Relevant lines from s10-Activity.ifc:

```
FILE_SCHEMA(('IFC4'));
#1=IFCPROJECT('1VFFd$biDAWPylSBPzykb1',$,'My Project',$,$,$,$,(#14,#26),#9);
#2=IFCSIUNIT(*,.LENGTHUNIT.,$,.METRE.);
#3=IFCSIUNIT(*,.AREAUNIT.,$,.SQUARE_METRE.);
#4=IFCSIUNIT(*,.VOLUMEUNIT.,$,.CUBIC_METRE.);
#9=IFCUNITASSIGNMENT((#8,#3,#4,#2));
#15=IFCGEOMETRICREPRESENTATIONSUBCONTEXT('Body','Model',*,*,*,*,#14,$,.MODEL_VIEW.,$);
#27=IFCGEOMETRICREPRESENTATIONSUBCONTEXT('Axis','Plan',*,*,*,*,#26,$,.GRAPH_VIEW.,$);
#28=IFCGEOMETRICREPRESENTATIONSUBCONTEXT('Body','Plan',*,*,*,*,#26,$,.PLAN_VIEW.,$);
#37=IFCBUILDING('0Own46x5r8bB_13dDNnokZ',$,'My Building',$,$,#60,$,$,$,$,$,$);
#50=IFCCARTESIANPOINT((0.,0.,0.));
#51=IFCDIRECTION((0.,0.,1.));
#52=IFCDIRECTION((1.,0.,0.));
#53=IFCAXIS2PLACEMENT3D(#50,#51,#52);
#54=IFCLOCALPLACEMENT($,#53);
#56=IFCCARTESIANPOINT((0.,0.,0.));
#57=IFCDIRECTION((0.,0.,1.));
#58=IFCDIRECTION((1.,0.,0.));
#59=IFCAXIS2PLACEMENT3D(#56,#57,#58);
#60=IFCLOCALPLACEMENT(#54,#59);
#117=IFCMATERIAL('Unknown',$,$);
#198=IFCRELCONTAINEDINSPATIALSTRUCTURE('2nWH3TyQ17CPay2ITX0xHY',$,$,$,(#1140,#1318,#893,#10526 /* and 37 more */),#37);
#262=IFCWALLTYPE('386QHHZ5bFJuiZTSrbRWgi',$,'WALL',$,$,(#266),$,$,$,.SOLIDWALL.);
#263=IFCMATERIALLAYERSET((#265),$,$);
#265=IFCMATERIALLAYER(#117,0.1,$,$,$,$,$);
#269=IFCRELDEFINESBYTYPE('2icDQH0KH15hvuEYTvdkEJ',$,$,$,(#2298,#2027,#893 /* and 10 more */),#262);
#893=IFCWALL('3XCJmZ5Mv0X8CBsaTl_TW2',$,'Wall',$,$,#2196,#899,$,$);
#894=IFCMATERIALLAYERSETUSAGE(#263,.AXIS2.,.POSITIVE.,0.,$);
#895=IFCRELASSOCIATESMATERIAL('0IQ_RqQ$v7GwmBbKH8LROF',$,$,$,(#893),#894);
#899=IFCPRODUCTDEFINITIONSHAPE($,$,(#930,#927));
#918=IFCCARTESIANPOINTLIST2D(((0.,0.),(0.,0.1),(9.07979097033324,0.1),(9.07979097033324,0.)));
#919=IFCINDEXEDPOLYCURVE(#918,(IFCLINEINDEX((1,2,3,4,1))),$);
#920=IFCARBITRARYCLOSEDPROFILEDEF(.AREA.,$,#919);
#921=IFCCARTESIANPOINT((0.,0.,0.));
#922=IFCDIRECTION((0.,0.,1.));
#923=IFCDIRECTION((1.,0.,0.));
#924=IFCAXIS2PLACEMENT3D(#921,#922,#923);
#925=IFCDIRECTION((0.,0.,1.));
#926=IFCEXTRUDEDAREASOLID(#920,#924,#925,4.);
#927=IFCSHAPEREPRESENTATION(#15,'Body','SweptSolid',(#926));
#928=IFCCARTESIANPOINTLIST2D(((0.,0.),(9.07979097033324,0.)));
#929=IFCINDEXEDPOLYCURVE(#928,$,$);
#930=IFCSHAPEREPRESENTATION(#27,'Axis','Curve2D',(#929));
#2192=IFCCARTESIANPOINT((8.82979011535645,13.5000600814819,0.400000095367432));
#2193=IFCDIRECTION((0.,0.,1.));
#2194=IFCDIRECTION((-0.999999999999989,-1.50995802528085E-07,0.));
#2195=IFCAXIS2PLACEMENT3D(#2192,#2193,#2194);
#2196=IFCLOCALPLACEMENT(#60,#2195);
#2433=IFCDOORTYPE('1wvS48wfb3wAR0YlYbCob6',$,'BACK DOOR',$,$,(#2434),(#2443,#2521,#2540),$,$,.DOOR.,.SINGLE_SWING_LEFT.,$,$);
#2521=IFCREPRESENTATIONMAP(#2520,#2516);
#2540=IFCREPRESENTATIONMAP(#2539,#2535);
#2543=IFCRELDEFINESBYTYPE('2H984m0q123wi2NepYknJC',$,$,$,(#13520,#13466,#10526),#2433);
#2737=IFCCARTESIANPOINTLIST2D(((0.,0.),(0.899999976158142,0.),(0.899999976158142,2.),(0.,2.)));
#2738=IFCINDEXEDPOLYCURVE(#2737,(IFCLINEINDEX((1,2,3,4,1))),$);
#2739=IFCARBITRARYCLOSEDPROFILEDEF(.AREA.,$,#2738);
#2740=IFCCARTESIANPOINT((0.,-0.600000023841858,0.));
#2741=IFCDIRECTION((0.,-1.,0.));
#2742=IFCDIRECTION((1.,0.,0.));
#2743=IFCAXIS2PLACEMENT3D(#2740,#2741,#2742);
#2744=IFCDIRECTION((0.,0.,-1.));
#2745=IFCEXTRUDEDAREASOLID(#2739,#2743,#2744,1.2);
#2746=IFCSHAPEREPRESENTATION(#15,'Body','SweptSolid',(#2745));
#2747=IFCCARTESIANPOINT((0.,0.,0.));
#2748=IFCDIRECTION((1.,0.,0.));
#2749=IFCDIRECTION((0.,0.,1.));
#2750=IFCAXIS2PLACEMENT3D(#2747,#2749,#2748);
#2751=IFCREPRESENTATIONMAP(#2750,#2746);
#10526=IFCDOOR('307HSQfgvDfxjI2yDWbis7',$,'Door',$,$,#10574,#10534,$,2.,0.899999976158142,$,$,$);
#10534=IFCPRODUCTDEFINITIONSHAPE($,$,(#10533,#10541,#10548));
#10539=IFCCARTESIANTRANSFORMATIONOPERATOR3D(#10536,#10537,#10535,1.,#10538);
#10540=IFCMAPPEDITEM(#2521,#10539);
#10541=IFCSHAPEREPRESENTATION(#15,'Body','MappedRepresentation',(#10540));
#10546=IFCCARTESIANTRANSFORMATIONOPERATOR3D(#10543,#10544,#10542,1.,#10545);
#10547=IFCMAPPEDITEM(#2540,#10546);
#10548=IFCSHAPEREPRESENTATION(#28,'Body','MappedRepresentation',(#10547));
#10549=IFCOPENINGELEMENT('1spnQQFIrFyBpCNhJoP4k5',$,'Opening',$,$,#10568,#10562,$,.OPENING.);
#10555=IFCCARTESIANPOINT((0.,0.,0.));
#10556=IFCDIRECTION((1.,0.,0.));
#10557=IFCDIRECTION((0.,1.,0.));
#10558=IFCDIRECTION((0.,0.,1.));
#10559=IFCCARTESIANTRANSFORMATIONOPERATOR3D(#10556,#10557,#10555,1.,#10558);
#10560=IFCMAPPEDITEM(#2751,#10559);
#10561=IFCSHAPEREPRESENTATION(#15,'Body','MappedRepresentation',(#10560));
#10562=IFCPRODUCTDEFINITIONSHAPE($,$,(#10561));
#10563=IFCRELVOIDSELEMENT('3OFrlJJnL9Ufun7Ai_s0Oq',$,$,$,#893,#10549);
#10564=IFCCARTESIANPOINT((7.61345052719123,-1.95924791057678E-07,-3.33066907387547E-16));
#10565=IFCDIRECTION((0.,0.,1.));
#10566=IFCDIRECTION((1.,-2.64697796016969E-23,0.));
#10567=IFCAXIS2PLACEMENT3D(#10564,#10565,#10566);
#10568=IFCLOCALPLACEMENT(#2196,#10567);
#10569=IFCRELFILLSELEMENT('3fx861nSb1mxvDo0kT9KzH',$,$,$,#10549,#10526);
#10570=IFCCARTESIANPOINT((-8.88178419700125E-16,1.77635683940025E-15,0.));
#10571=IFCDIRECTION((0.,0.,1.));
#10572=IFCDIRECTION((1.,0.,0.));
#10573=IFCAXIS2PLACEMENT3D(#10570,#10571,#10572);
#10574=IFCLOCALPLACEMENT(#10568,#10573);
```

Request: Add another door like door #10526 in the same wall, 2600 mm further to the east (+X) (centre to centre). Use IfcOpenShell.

```python
import ifcopenshell
import ifcopenshell.api.feature
import ifcopenshell.api.geometry
import ifcopenshell.api.root
import ifcopenshell.geom
import ifcopenshell.util.element
import ifcopenshell.util.placement
import ifcopenshell.util.shape

model = ifcopenshell.open("s10-Activity.ifc")
settings = ifcopenshell.geom.settings()


def volume(element):
    """Net volume in cubic metres, openings subtracted."""
    shape = ifcopenshell.geom.create_shape(settings, element)
    return ifcopenshell.util.shape.get_volume(shape.geometry)


door = model.by_guid("307HSQfgvDfxjI2yDWbis7")
opening = door.FillsVoids[0].RelatingOpeningElement
wall = opening.VoidsElements[0].RelatingBuildingElement
before = volume(wall)
shift = ifcopenshell.util.placement.get_local_placement(wall.ObjectPlacement)[:3, 0] * -2.6

# copy_class copies the void relationship, type, container and properties, but no geometry.
new_opening = ifcopenshell.api.root.copy_class(model, product=opening)
new_opening.Representation = ifcopenshell.util.element.copy_deep(
    model, opening.Representation, exclude=["IfcGeometricRepresentationContext", "IfcRepresentationMap"]
)
new_door = ifcopenshell.api.root.copy_class(model, product=door)
new_door.Representation = ifcopenshell.util.element.copy_deep(
    model, door.Representation, exclude=["IfcGeometricRepresentationContext", "IfcRepresentationMap"]
)
ifcopenshell.api.feature.add_filling(model, opening=new_opening, element=new_door)

for old, new in ((opening, new_opening), (door, new_door)):
    matrix = ifcopenshell.util.placement.get_local_placement(old.ObjectPlacement)
    matrix[:3, 3] += shift
    ifcopenshell.api.geometry.edit_object_placement(model, product=new, matrix=matrix, is_si=False)

after = volume(wall)

print(f"wall volume {before:.3f} -> {after:.3f} m3")

model.write("s10-Activity_rev.ifc")
```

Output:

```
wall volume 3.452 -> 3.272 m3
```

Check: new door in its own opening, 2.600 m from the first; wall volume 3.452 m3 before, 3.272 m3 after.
